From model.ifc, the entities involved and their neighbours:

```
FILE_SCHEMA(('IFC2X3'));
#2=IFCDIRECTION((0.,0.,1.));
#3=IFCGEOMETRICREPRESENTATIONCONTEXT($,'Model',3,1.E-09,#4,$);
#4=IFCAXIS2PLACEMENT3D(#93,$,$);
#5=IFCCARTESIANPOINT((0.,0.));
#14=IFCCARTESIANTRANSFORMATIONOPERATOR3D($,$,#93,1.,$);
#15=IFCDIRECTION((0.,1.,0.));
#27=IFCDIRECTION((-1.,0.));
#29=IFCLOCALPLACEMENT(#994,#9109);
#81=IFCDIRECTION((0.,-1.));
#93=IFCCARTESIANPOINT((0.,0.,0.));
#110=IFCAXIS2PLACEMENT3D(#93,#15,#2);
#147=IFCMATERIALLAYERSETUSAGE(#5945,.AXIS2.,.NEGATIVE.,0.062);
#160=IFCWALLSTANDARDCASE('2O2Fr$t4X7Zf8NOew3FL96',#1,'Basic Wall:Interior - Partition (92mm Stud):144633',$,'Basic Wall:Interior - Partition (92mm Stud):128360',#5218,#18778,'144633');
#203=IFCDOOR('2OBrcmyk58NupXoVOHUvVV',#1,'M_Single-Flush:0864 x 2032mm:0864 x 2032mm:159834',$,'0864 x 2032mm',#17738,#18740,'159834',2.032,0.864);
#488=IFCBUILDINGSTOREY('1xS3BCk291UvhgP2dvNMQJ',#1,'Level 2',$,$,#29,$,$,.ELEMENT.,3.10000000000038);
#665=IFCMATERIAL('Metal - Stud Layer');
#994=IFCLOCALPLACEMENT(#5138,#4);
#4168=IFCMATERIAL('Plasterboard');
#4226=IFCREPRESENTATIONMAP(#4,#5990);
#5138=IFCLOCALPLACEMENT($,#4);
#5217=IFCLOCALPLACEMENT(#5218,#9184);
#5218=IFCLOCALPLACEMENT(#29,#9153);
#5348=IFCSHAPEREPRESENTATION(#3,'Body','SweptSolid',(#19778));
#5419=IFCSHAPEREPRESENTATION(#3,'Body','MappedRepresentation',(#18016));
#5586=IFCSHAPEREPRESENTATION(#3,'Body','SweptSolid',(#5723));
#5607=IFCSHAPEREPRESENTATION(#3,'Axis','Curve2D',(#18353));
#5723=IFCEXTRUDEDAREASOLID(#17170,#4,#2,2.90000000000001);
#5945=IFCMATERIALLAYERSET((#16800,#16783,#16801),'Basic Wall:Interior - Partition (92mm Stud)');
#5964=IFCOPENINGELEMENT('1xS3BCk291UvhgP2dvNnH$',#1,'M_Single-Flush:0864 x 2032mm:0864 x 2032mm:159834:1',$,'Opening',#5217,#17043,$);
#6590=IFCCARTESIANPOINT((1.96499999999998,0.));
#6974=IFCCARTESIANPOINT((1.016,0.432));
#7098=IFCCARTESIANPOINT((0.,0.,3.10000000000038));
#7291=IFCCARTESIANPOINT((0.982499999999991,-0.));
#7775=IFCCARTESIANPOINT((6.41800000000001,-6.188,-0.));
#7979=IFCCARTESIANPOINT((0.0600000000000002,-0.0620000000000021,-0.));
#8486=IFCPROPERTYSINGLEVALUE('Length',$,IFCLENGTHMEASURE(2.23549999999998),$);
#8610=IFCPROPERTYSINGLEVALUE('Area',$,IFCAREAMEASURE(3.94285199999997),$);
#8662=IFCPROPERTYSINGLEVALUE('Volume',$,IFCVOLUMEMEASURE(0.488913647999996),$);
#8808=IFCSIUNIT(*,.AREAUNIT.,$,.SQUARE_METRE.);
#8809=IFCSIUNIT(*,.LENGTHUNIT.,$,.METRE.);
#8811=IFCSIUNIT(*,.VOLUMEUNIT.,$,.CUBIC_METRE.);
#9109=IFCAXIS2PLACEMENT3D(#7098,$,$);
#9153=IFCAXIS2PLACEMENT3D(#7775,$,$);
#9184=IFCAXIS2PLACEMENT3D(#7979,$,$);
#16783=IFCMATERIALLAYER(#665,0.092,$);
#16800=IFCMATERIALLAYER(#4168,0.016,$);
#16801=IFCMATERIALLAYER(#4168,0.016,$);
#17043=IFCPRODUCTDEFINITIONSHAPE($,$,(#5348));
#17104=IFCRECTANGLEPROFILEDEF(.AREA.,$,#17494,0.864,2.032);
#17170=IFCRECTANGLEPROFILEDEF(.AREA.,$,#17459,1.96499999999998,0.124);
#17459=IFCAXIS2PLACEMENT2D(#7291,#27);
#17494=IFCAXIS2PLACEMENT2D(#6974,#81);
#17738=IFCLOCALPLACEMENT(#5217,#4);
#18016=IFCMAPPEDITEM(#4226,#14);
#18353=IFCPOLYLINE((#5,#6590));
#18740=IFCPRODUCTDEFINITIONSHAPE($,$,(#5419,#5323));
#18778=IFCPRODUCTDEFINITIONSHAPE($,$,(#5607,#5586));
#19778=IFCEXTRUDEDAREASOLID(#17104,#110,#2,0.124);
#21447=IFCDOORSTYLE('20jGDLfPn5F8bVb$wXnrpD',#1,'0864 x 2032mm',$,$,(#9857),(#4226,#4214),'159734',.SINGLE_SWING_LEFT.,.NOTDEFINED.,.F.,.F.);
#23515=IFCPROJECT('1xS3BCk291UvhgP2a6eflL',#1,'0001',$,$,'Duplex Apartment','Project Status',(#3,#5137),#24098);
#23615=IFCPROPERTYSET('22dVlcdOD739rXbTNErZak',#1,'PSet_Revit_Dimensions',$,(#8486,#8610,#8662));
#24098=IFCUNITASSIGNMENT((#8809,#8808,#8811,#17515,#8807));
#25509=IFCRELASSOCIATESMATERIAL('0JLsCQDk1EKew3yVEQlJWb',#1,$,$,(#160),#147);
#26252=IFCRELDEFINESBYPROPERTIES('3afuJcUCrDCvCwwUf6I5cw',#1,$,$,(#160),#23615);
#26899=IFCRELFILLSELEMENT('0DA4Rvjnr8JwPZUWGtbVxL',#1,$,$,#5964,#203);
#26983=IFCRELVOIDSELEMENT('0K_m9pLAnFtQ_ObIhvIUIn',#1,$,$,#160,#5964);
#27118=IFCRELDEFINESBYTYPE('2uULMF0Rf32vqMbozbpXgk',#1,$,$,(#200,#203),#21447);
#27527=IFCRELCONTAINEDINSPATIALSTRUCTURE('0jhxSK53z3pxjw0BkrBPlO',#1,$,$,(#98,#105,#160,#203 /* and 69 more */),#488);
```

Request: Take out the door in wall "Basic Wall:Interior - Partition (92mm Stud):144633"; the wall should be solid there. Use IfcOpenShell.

```python
import ifcopenshell
import ifcopenshell.api.feature
import ifcopenshell.api.pset
import ifcopenshell.api.root
import ifcopenshell.geom
import ifcopenshell.util.element
import ifcopenshell.util.shape
import ifcopenshell.util.unit

model = ifcopenshell.open("model.ifc")
area_scale = ifcopenshell.util.unit.calculate_unit_scale(model, "AREAUNIT")
volume_scale = ifcopenshell.util.unit.calculate_unit_scale(model, "VOLUMEUNIT")
settings = ifcopenshell.geom.settings()


def volume(element):
    """Net volume in cubic metres, openings subtracted."""
    shape = ifcopenshell.geom.create_shape(settings, element)
    return ifcopenshell.util.shape.get_volume(shape.geometry)


door = model.by_guid("2OBrcmyk58NupXoVOHUvVV")
opening = door.FillsVoids[0].RelatingOpeningElement
wall = opening.VoidsElements[0].RelatingBuildingElement
before = volume(wall)

ifcopenshell.api.root.remove_product(model, product=door)
ifcopenshell.api.feature.remove_feature(model, feature=opening)

after = volume(wall)
thickness = 0.124  # wall thickness in metres

# Update the wall's stored quantities.
pset = model.by_id(ifcopenshell.util.element.get_pset(wall, "PSet_Revit_Dimensions", should_inherit=False)["id"])
ifcopenshell.api.pset.edit_pset(model, pset=pset, properties={
    "Area": model.create_entity("IfcAreaMeasure", after / thickness / area_scale),
    "Volume": model.create_entity("IfcVolumeMeasure", after / volume_scale),
})

print(f"wall volume {before:.3f} -> {after:.3f} m3")

model.write("model_updated.ifc")
```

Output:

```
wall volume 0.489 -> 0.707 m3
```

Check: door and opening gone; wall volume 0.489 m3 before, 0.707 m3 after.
